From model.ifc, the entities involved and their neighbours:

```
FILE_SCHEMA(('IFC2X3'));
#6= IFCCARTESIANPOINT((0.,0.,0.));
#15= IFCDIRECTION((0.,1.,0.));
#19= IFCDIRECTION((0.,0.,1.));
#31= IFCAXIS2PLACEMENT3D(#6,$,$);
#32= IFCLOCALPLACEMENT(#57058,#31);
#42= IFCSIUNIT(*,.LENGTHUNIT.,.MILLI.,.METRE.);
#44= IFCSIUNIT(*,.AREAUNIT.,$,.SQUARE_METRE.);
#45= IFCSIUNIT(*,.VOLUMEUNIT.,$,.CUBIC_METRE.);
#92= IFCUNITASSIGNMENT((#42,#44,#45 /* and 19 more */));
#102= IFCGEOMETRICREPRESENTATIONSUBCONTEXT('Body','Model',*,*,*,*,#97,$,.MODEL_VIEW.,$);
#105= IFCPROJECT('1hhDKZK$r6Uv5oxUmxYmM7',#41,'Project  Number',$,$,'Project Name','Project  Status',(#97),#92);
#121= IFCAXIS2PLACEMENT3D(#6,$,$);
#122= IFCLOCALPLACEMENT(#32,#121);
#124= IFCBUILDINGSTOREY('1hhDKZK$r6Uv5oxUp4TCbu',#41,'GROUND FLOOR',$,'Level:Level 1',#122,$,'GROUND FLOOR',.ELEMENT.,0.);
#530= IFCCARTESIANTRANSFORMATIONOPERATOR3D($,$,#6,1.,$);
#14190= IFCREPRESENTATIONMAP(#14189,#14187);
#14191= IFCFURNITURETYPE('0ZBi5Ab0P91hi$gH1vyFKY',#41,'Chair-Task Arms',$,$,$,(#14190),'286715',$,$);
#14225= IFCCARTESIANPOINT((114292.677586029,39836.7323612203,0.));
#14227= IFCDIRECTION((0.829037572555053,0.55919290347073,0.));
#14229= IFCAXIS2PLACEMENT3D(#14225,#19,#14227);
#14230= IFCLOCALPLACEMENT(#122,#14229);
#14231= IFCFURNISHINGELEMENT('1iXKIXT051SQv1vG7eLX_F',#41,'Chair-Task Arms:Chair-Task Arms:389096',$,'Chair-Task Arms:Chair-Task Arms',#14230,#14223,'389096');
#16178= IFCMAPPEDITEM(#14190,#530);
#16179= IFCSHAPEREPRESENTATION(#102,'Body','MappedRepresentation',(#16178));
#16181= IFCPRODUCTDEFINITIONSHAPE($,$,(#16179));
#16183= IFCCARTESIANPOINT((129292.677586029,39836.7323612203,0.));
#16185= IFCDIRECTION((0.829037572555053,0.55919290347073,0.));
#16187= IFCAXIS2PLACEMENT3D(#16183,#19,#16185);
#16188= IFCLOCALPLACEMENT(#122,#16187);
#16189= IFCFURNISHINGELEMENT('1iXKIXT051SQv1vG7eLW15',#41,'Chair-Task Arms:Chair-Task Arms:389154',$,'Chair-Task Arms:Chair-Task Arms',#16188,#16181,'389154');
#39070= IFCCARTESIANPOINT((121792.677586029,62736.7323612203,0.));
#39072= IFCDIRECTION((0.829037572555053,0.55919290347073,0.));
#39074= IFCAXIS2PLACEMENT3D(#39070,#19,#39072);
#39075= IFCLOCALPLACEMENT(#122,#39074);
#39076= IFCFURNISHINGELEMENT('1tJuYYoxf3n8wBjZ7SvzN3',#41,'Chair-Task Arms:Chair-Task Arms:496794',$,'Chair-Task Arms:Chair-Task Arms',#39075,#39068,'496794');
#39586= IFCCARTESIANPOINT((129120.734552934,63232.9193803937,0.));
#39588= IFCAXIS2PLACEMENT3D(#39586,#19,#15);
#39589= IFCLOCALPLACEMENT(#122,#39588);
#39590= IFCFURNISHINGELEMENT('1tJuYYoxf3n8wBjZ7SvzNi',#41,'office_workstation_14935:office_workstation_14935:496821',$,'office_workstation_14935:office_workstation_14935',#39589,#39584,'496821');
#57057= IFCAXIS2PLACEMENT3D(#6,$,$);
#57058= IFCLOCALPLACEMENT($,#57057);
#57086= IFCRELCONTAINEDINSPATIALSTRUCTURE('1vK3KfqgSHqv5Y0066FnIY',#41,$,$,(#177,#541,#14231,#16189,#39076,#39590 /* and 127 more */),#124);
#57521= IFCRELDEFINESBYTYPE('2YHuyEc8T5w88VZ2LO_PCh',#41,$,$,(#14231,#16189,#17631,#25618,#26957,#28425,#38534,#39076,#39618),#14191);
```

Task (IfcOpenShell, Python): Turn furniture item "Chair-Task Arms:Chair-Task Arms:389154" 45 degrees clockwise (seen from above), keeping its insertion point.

```python
import ifcopenshell
import ifcopenshell.api.geometry
import ifcopenshell.util.placement

model = ifcopenshell.open("model.ifc")

item = model.by_guid("1iXKIXT051SQv1vG7eLW15")
matrix = ifcopenshell.util.placement.get_local_placement(item.ObjectPlacement)
matrix = matrix @ ifcopenshell.util.placement.rotation(-45, "Z")
ifcopenshell.api.geometry.edit_object_placement(model, product=item, matrix=matrix, is_si=False)

print(ifcopenshell.util.placement.get_local_placement(item.ObjectPlacement).round(3) + 0.0)

model.write("model-out.ifc")
```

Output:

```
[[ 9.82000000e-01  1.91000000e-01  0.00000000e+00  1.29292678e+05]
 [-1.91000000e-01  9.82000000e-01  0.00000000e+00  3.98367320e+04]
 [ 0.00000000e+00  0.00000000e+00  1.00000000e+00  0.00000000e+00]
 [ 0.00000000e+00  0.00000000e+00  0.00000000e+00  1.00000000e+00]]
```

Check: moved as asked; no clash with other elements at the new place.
